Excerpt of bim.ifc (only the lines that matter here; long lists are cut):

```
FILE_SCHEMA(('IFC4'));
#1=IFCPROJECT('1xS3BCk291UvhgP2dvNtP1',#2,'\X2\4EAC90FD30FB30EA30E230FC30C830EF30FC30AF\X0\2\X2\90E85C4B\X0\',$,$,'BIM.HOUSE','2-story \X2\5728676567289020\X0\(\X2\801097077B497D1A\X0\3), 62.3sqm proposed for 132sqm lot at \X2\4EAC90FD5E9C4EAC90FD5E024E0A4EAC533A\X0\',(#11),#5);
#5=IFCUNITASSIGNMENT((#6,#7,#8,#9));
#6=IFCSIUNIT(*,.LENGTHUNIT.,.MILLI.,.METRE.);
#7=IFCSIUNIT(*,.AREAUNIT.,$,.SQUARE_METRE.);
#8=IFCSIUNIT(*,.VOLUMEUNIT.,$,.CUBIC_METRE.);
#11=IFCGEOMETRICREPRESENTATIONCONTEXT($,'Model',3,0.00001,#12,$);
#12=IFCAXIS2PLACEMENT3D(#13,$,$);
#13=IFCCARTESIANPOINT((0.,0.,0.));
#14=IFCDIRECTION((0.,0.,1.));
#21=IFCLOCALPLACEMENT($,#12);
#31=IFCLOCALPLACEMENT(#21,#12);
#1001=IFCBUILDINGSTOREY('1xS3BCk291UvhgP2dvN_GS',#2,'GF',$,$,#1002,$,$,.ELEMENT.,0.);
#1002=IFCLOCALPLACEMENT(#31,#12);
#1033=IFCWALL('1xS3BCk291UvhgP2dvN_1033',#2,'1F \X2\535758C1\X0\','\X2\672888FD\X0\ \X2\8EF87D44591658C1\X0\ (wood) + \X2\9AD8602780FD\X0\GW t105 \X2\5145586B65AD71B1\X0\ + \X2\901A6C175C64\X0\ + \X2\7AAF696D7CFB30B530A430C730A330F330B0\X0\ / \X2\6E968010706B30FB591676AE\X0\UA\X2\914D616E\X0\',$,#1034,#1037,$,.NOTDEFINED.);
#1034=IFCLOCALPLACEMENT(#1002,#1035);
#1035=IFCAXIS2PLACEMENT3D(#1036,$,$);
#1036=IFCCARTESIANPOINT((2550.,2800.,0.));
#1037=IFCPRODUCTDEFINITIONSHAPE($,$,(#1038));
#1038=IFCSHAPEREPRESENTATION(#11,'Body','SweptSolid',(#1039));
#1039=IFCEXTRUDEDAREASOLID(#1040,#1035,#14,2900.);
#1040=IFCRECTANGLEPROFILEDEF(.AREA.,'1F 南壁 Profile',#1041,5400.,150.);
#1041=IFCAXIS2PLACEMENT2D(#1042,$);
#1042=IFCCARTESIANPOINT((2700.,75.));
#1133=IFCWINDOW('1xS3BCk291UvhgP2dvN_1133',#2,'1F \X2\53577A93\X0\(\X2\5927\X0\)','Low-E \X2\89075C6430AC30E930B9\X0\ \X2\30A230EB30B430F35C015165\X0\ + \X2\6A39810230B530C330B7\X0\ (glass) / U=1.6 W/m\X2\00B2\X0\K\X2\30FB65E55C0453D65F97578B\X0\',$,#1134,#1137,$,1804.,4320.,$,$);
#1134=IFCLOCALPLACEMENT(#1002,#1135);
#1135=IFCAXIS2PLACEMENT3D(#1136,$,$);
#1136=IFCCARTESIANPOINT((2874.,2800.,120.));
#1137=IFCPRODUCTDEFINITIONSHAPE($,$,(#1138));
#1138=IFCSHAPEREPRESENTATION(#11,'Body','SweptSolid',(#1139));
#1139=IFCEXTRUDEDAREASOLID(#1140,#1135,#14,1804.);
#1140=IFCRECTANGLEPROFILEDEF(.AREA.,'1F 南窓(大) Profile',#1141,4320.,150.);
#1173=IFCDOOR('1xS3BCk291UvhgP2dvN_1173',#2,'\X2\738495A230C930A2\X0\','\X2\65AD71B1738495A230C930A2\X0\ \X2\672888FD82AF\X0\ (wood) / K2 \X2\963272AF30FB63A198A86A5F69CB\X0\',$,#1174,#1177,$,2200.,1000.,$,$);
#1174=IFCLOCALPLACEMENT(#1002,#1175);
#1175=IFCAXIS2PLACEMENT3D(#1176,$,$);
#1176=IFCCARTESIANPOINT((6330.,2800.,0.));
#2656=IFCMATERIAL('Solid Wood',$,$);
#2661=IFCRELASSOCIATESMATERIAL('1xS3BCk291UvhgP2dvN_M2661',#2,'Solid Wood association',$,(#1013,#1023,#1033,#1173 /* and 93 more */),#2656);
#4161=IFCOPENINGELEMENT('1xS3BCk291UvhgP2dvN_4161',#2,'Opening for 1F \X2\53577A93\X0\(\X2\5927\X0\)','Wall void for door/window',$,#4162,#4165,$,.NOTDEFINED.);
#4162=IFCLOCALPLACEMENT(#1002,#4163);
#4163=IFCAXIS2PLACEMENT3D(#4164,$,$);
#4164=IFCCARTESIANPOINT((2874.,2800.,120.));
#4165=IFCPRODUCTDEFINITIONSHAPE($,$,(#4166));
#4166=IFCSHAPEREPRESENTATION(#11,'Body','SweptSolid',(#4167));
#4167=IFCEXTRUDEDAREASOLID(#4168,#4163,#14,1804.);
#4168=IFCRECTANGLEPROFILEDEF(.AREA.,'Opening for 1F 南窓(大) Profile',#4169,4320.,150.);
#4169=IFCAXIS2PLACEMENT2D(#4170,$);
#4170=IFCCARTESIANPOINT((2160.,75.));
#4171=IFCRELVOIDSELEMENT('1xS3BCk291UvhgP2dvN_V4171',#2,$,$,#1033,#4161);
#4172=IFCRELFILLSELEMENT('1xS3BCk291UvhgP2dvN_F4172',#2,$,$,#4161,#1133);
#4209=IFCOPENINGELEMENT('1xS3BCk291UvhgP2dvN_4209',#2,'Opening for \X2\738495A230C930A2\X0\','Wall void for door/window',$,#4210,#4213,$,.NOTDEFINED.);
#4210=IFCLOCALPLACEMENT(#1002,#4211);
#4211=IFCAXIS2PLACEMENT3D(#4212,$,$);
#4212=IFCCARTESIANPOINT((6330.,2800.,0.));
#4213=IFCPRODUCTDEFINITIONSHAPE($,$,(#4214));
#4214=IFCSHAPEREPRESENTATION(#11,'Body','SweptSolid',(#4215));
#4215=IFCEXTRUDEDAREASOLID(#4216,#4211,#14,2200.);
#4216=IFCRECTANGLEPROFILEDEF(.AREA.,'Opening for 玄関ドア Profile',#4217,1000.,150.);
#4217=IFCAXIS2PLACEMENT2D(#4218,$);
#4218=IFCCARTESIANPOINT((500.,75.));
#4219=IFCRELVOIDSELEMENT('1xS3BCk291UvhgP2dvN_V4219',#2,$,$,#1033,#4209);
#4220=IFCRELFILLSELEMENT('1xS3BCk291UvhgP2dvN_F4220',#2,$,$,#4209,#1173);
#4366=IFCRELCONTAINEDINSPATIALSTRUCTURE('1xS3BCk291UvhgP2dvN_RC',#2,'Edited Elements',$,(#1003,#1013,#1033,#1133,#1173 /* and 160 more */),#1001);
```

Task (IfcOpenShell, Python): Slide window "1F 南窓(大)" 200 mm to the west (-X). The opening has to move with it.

```python
import ifcopenshell
import ifcopenshell.api.geometry
import ifcopenshell.util.placement

model = ifcopenshell.open("bim.ifc")

window = model.by_guid("1xS3BCk291UvhgP2dvN_1133")
opening = window.FillsVoids[0].RelatingOpeningElement
wall = opening.VoidsElements[0].RelatingBuildingElement

wall_matrix = ifcopenshell.util.placement.get_local_placement(wall.ObjectPlacement)
shift = wall_matrix[:3, 0] * -200.0
before = ifcopenshell.util.placement.get_local_placement(window.ObjectPlacement)[:3, 3].copy()

# The window is not placed relative to its opening, so move both.
for product in (opening, window):
    matrix = ifcopenshell.util.placement.get_local_placement(product.ObjectPlacement)
    matrix[:3, 3] += shift
    ifcopenshell.api.geometry.edit_object_placement(model, product=product, matrix=matrix, is_si=False)

after = ifcopenshell.util.placement.get_local_placement(window.ObjectPlacement)[:3, 3]
print("window moved by", (after - before).round(3) + 0.0)

model.write("bim_v2.ifc")
```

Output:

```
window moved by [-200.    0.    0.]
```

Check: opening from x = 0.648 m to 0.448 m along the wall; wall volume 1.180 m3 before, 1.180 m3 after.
